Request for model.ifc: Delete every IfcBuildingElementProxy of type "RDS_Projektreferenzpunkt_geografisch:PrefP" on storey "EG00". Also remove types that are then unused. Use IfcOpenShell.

First a look at what the model holds.

```python
import ifcopenshell
import ifcopenshell.util.element

model = ifcopenshell.open("model.ifc")
print(model.schema)
storey = next(s for s in model.by_type("IfcBuildingStorey") if s.Name == "EG00")
proxies = [e for e in ifcopenshell.util.element.get_decomposition(storey) if e.is_a("IfcBuildingElementProxy")]
seen = {}
for e in proxies:
    element_type = ifcopenshell.util.element.get_type(e)
    name = element_type.Name if element_type not in (None, e) else None
    seen[name] = seen.get(name, 0) + 1
for name, count in sorted(seen.items(), key=str):
    print(count, "x", name)
```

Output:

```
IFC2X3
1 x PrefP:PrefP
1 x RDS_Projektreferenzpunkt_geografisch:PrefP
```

```python
import ifcopenshell
import ifcopenshell.api.root
import ifcopenshell.util.element

model = ifcopenshell.open("model.ifc")

storey = next(s for s in model.by_type("IfcBuildingStorey") if s.Name == "EG00")
proxies = [e for e in ifcopenshell.util.element.get_decomposition(storey) if e.is_a("IfcBuildingElementProxy")]
targets = [e for e in proxies if (t := ifcopenshell.util.element.get_type(e)) not in (None, e) and t.Name == "RDS_Projektreferenzpunkt_geografisch:PrefP"]
types = {ifcopenshell.util.element.get_type(e) for e in targets} - {None, *targets}

for e in targets:
    ifcopenshell.api.root.remove_product(model, product=e)
print(len(targets), "removed")

unused = [t for t in types if not ifcopenshell.util.element.get_types(t)]
for t in unused:
    ifcopenshell.api.root.remove_product(model, product=t)
print(len(unused), "unused types removed")

model.write("model-out.ifc")
```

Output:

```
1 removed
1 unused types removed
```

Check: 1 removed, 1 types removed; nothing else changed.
